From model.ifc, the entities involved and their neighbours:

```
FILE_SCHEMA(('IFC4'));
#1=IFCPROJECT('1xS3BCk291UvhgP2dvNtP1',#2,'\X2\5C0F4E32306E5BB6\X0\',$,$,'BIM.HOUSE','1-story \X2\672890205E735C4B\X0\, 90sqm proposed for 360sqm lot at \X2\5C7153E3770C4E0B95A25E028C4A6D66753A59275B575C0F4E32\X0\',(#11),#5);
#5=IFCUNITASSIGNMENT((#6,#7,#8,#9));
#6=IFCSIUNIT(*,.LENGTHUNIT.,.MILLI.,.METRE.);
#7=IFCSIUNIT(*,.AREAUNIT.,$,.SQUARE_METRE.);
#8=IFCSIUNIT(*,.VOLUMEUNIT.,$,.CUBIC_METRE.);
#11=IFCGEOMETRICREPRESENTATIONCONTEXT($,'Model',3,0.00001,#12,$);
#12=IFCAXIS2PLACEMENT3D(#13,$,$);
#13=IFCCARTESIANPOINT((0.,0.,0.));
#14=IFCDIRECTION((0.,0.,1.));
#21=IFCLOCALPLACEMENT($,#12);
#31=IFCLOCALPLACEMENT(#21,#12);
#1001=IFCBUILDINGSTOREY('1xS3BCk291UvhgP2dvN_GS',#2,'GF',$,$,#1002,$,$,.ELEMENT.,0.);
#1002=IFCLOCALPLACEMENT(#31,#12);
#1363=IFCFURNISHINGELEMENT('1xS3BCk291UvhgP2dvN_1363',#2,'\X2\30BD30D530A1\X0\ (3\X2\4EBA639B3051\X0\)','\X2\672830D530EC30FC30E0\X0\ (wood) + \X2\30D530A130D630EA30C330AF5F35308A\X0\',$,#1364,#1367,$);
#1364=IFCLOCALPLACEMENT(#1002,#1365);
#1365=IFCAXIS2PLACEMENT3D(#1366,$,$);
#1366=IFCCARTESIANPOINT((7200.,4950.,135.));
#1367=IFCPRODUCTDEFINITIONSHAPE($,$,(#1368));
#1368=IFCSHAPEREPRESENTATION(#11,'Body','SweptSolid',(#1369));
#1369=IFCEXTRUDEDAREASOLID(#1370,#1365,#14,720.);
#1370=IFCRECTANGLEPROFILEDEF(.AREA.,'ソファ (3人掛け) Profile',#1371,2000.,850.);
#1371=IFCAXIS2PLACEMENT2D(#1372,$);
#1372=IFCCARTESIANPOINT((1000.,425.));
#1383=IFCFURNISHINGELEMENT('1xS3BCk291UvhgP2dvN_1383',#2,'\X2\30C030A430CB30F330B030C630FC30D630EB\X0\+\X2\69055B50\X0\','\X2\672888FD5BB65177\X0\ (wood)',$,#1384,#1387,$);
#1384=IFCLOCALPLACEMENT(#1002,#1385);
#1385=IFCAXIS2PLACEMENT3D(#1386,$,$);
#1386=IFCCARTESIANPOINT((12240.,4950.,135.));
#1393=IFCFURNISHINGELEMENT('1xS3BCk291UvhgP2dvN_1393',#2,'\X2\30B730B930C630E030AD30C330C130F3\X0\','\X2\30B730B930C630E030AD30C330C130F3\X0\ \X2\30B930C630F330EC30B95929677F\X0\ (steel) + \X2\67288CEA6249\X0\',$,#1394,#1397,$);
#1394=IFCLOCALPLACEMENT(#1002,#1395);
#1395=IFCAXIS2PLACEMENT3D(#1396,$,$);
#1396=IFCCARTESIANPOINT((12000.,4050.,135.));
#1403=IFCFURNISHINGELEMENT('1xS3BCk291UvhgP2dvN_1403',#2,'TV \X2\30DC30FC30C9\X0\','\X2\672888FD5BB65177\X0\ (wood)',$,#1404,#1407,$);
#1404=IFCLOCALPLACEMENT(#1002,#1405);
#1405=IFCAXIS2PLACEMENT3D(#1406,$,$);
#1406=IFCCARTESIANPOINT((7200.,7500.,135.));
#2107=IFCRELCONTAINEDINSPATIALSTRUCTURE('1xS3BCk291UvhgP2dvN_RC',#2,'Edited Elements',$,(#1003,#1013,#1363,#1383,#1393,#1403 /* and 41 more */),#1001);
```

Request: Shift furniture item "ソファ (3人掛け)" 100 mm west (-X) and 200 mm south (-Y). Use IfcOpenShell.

```python
import ifcopenshell
import ifcopenshell.api.geometry
import ifcopenshell.util.placement

model = ifcopenshell.open("model.ifc")

item = model.by_id(1363)
matrix = ifcopenshell.util.placement.get_local_placement(item.ObjectPlacement)
matrix[0, 3] -= 100.0
matrix[1, 3] -= 200.0
ifcopenshell.api.geometry.edit_object_placement(model, product=item, matrix=matrix, is_si=False)

print(ifcopenshell.util.placement.get_local_placement(item.ObjectPlacement).round(3) + 0.0)

model.write("model_v2.ifc")
```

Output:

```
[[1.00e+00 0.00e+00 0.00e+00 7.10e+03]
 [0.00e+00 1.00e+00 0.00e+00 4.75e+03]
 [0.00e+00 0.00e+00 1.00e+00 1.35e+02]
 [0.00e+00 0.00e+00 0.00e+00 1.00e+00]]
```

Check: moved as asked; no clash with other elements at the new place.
